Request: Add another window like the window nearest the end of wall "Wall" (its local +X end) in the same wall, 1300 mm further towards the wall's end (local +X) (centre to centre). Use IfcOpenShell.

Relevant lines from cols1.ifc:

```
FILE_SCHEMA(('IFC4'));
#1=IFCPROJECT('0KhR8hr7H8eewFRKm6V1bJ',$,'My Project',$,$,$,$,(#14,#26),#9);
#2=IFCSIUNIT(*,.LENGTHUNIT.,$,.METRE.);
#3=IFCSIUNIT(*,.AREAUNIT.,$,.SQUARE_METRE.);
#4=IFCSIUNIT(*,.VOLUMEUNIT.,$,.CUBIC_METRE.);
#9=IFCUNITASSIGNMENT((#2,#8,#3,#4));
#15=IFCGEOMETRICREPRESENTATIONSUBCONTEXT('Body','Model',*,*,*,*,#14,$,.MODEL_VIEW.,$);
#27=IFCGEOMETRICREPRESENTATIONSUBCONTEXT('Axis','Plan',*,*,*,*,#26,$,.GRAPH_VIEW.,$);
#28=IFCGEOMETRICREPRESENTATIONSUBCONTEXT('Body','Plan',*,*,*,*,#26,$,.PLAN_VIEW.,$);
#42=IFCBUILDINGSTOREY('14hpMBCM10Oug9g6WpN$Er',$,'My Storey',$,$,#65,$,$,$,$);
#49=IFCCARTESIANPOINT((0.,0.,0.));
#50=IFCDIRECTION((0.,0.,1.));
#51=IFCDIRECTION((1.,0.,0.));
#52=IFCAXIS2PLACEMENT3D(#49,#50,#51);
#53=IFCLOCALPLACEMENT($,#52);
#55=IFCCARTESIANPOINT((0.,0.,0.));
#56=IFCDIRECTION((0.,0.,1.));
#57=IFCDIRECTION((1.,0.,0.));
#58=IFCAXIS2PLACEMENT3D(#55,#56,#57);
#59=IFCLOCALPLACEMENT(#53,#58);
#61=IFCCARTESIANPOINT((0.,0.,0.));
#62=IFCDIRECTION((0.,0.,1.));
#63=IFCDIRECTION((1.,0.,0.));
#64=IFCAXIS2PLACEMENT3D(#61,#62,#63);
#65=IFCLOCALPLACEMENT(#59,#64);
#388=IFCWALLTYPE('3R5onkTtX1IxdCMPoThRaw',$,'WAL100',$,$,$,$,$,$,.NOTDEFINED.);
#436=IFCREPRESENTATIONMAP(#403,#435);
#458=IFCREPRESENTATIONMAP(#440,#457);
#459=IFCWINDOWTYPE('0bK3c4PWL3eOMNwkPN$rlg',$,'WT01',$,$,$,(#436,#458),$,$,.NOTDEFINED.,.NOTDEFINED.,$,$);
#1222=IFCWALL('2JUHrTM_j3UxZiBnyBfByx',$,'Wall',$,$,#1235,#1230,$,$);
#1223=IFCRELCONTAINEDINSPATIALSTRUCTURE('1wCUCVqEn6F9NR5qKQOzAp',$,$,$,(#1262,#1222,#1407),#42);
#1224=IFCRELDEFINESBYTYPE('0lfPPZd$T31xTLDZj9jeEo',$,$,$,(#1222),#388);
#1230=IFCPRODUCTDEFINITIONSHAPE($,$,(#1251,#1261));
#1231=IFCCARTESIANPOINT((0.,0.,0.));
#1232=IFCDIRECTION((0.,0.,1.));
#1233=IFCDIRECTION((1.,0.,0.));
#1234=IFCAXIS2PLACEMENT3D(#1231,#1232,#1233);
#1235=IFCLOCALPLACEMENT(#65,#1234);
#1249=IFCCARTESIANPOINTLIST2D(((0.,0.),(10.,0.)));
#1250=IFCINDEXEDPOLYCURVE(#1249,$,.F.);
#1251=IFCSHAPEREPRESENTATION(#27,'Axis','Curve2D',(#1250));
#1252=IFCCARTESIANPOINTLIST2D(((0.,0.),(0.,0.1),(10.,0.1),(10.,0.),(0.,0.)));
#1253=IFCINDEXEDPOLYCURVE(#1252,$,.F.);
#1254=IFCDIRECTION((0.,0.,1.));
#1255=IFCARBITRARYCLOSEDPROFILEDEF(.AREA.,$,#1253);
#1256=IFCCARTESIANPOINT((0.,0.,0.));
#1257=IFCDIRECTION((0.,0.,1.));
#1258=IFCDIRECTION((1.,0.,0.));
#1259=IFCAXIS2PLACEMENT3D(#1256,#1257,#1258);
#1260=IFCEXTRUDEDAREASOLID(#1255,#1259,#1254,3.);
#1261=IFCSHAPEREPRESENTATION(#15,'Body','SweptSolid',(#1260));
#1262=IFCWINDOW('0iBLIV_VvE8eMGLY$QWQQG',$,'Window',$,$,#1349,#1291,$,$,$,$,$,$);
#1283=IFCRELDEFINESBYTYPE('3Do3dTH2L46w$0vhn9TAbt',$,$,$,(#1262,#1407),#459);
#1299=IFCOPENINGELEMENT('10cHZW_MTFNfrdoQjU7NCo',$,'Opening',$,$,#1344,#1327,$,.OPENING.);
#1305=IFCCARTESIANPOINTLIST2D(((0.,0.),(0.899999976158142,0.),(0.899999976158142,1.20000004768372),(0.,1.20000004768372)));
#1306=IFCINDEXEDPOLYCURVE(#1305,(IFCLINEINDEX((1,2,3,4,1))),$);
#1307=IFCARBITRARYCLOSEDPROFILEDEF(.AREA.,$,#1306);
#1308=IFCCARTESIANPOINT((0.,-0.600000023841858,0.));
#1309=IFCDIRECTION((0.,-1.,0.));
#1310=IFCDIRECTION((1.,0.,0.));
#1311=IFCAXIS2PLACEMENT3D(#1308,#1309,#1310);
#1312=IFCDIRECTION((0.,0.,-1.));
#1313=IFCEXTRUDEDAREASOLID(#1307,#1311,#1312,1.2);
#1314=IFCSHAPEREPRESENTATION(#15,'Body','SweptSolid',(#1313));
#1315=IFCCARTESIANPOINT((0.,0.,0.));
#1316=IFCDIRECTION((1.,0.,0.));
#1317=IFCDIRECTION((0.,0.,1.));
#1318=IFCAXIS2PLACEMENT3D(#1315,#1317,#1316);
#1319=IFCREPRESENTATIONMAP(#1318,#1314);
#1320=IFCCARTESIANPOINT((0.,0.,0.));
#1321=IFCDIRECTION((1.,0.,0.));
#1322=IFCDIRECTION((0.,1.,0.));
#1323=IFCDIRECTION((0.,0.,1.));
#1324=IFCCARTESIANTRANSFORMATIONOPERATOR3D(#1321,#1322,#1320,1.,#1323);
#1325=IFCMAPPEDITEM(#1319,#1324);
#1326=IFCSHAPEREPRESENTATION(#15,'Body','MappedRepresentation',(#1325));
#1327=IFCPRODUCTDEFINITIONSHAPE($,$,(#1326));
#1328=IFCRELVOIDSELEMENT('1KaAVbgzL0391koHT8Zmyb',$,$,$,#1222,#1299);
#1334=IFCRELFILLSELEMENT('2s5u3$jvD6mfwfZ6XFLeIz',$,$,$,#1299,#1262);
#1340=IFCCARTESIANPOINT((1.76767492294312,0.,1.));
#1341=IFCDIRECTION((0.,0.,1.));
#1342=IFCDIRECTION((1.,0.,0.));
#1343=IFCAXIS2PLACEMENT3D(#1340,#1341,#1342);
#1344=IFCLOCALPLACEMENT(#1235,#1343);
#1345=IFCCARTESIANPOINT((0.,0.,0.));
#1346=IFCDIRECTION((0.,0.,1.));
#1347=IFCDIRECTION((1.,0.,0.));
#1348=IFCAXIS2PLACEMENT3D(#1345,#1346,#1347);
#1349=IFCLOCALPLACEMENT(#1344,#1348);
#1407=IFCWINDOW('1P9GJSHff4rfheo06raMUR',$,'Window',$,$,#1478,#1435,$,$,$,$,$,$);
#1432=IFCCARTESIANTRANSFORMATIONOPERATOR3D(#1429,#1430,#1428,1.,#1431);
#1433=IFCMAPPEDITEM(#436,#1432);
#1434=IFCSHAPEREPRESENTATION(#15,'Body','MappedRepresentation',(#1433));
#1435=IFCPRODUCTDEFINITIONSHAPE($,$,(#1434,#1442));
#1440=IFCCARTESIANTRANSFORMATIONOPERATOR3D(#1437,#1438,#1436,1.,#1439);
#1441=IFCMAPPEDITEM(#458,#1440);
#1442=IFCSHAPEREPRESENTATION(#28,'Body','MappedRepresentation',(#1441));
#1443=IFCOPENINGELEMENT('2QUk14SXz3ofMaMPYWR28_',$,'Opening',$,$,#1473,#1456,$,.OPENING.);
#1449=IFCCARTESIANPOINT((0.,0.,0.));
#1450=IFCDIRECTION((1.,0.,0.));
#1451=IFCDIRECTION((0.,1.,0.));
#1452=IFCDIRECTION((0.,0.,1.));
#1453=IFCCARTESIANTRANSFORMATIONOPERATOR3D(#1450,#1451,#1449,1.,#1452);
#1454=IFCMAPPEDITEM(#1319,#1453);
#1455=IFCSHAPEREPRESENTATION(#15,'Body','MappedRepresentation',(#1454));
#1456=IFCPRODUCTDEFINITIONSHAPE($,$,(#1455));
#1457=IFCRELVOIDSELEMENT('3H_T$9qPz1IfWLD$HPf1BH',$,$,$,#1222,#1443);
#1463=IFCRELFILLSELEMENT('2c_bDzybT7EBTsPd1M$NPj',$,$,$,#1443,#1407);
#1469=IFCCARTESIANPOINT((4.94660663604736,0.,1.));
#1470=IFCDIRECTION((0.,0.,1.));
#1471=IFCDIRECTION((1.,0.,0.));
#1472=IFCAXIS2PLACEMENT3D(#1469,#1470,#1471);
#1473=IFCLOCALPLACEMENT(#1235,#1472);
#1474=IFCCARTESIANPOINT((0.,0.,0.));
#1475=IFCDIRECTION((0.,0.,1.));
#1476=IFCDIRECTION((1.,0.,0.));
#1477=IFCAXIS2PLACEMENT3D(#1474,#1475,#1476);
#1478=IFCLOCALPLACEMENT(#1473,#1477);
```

```python
import ifcopenshell
import ifcopenshell.api.feature
import ifcopenshell.api.geometry
import ifcopenshell.api.root
import ifcopenshell.geom
import ifcopenshell.util.element
import ifcopenshell.util.placement
import ifcopenshell.util.shape

model = ifcopenshell.open("cols1.ifc")
settings = ifcopenshell.geom.settings()


def volume(element):
    """Net volume in cubic metres, openings subtracted."""
    shape = ifcopenshell.geom.create_shape(settings, element)
    return ifcopenshell.util.shape.get_volume(shape.geometry)


window = model.by_guid("1P9GJSHff4rfheo06raMUR")
opening = window.FillsVoids[0].RelatingOpeningElement
wall = opening.VoidsElements[0].RelatingBuildingElement
before = volume(wall)
shift = ifcopenshell.util.placement.get_local_placement(wall.ObjectPlacement)[:3, 0] * 1.3

# copy_class copies the void relationship, type, container and properties, but no geometry.
new_opening = ifcopenshell.api.root.copy_class(model, product=opening)
new_opening.Representation = ifcopenshell.util.element.copy_deep(
    model, opening.Representation, exclude=["IfcGeometricRepresentationContext", "IfcRepresentationMap"]
)
new_window = ifcopenshell.api.root.copy_class(model, product=window)
new_window.Representation = ifcopenshell.util.element.copy_deep(
    model, window.Representation, exclude=["IfcGeometricRepresentationContext", "IfcRepresentationMap"]
)
ifcopenshell.api.feature.add_filling(model, opening=new_opening, element=new_window)

for old, new in ((opening, new_opening), (window, new_window)):
    matrix = ifcopenshell.util.placement.get_local_placement(old.ObjectPlacement)
    matrix[:3, 3] += shift
    ifcopenshell.api.geometry.edit_object_placement(model, product=new, matrix=matrix, is_si=False)

after = volume(wall)

print(f"wall volume {before:.3f} -> {after:.3f} m3")

model.write("cols1_rev.ifc")
```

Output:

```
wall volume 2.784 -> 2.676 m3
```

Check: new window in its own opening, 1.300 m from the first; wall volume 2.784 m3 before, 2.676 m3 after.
